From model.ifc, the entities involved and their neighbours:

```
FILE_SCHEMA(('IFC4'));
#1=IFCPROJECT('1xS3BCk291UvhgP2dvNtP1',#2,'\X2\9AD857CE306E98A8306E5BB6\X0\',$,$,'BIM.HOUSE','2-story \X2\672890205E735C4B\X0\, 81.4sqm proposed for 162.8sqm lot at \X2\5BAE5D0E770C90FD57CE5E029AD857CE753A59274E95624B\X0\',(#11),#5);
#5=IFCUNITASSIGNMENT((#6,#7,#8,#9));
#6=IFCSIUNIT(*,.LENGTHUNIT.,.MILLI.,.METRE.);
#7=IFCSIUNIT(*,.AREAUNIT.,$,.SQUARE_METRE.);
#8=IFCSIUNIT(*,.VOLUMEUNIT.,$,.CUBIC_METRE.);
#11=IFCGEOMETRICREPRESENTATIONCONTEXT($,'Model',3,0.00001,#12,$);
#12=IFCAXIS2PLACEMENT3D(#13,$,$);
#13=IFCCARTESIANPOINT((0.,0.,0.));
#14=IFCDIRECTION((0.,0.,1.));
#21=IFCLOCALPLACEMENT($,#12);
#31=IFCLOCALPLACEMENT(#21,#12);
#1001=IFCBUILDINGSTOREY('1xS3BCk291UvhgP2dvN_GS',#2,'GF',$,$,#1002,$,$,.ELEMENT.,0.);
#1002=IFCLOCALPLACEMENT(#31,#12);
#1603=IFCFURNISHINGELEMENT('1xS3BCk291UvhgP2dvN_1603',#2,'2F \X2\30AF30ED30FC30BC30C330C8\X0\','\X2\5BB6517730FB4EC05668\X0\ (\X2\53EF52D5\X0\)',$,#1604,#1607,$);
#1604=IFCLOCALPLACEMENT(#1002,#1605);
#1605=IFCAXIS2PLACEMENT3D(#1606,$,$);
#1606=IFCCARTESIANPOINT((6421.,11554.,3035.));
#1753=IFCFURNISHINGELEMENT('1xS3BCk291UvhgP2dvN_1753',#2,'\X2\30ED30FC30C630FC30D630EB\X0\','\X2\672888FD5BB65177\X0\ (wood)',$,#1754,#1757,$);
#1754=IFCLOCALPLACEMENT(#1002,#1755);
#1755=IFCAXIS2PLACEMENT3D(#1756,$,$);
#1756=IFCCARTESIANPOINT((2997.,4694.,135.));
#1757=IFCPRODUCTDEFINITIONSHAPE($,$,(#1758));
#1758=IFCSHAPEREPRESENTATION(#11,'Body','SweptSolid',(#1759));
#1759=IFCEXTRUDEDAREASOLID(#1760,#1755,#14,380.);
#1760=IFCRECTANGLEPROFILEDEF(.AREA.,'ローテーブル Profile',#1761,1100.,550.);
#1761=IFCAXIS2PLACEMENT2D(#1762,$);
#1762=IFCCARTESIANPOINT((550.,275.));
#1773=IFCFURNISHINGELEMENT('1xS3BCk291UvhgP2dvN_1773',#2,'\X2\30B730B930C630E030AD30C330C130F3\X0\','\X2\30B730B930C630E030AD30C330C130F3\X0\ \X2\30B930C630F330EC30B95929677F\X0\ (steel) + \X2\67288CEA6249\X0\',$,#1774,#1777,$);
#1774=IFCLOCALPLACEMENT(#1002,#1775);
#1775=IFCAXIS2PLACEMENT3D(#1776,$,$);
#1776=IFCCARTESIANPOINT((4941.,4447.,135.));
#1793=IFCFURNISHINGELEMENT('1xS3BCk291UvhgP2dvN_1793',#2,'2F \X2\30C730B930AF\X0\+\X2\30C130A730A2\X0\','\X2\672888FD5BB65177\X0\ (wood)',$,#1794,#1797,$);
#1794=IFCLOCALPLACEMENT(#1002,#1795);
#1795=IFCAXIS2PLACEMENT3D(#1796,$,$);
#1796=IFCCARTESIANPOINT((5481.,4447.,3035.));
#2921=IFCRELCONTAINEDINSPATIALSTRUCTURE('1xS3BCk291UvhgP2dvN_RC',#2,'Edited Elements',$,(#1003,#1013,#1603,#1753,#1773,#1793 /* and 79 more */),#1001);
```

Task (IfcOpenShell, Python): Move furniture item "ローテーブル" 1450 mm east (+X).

```python
import ifcopenshell
import ifcopenshell.api.geometry
import ifcopenshell.util.placement
import ifcopenshell.util.unit

model = ifcopenshell.open("model.ifc")
unit_scale = ifcopenshell.util.unit.calculate_unit_scale(model)

item = model.by_guid("1xS3BCk291UvhgP2dvN_1753")
matrix = ifcopenshell.util.placement.get_local_placement(item.ObjectPlacement)
matrix[0, 3] += 1.45 / unit_scale
ifcopenshell.api.geometry.edit_object_placement(model, product=item, matrix=matrix, is_si=False)

print(ifcopenshell.util.placement.get_local_placement(item.ObjectPlacement).round(3) + 0.0)

model.write("model_edited.ifc")
```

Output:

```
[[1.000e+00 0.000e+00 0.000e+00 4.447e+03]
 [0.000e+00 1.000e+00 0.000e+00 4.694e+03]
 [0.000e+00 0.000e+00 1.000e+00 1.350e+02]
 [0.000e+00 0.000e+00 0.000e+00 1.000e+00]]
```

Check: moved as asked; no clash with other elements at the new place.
